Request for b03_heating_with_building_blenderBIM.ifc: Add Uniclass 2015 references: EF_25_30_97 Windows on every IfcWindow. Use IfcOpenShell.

First a look at what the model holds.

```python
import ifcopenshell

model = ifcopenshell.open("b03_heating_with_building_blenderBIM.ifc")
print(model.schema)
print("classifications:", [c.Name for c in model.by_type("IfcClassification")])
for ifc_class in ("IfcDoor", "IfcRoof", "IfcStair", "IfcWall", "IfcWindow"):
    print(ifc_class, len(model.by_type(ifc_class)))
```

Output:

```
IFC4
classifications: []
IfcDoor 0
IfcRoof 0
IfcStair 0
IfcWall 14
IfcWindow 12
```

```python
import ifcopenshell
import ifcopenshell.api.classification

model = ifcopenshell.open("b03_heating_with_building_blenderBIM.ifc")

system = ifcopenshell.api.classification.add_classification(model, classification="Uniclass 2015")

codes = {
    "IfcWindow": ("EF_25_30_97", "Windows"),
}
for ifc_class, (code, name) in codes.items():
    products = model.by_type(ifc_class)
    ifcopenshell.api.classification.add_reference(
        model, products=products, classification=system, identification=code, name=name
    )
    print(code, len(products))

model.write("b03_heating_with_building_blenderBIM_rev.ifc")
```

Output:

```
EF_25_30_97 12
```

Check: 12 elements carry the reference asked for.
